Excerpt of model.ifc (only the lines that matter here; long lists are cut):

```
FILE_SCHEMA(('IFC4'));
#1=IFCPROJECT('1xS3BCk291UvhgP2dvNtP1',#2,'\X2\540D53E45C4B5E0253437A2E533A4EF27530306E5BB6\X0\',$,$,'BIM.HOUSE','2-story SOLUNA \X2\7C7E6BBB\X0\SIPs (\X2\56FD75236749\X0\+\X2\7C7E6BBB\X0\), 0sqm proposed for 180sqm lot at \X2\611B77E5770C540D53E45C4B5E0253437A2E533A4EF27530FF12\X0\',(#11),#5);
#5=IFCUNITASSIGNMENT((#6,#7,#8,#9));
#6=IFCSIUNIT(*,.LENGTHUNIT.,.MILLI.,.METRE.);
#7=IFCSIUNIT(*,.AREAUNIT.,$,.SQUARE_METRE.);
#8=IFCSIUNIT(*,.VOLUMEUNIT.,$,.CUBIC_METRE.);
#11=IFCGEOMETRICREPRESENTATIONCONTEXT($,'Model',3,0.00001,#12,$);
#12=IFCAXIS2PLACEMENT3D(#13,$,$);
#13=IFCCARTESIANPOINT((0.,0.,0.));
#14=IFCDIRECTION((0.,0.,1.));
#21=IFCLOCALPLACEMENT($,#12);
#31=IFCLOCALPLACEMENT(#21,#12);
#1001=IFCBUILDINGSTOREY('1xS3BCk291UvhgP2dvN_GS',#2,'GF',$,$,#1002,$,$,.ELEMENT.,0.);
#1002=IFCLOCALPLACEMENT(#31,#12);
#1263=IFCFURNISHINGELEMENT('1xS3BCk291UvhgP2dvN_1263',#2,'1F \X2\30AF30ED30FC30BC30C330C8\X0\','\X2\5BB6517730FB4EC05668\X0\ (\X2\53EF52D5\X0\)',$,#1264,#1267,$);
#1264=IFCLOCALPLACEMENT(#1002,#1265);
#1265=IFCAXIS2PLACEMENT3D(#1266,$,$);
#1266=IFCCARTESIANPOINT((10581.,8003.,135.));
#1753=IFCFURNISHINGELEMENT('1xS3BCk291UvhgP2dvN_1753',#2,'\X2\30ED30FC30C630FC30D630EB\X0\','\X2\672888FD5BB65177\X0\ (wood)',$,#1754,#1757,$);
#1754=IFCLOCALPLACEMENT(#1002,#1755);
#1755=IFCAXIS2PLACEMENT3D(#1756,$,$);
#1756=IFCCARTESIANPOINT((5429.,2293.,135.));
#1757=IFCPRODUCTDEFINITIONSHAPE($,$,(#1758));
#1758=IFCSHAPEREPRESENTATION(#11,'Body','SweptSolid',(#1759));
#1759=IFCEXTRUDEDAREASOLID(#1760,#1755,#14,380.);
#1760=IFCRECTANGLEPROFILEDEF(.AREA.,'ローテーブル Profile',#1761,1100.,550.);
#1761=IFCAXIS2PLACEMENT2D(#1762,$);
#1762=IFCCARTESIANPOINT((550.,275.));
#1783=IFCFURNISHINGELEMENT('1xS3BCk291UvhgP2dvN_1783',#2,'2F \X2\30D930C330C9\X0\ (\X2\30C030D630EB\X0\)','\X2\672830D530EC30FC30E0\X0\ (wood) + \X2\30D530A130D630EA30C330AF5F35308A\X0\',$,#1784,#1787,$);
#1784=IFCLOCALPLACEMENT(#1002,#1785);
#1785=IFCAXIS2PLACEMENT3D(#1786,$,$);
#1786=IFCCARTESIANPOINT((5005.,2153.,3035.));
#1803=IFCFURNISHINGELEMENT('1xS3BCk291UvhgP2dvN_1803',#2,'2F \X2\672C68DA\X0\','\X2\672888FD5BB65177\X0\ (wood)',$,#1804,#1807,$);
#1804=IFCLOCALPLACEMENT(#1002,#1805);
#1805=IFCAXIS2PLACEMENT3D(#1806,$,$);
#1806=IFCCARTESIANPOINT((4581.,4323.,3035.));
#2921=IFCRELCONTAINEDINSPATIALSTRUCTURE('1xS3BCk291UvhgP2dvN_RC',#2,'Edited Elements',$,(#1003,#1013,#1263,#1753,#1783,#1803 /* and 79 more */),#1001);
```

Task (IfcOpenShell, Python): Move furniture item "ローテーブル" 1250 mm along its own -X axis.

```python
import ifcopenshell
import ifcopenshell.api.geometry
import ifcopenshell.util.placement
import ifcopenshell.util.unit

model = ifcopenshell.open("model.ifc")
unit_scale = ifcopenshell.util.unit.calculate_unit_scale(model)

item = model.by_id(1753)
matrix = ifcopenshell.util.placement.get_local_placement(item.ObjectPlacement)
matrix[:3, 3] -= matrix[:3, 0] * 1.25 / unit_scale
ifcopenshell.api.geometry.edit_object_placement(model, product=item, matrix=matrix, is_si=False)

print(ifcopenshell.util.placement.get_local_placement(item.ObjectPlacement).round(3) + 0.0)

model.write("model_rev.ifc")
```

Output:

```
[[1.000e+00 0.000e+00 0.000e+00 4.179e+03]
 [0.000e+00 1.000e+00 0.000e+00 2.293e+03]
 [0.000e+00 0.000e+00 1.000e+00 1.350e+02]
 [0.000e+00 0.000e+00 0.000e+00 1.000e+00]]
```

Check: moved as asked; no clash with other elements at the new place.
